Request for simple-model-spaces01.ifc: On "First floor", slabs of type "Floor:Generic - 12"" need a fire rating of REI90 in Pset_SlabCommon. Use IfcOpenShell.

First a look at what the model holds.

```python
import ifcopenshell
import ifcopenshell.util.element

model = ifcopenshell.open("simple-model-spaces01.ifc")
print(model.schema)
storey = next(s for s in model.by_type("IfcBuildingStorey") if s.Name == "First floor")
slabs = [e for e in ifcopenshell.util.element.get_decomposition(storey) if e.is_a("IfcSlab")]
seen = {}
for e in slabs:
    element_type = ifcopenshell.util.element.get_type(e)
    key = (element_type.Name if element_type != e and element_type else None, ifcopenshell.util.element.get_pset(e, "Pset_SlabCommon", "FireRating"))
    seen[key] = seen.get(key, 0) + 1
for (name, value), count in sorted(seen.items(), key=str):
    print(count, "x", name, "|", value)
```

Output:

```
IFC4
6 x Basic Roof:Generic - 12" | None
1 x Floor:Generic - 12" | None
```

```python
import ifcopenshell
import ifcopenshell.api.pset
import ifcopenshell.util.element

model = ifcopenshell.open("simple-model-spaces01.ifc")

storey = next(s for s in model.by_type("IfcBuildingStorey") if s.Name == "First floor")
slabs = [e for e in ifcopenshell.util.element.get_decomposition(storey) if e.is_a("IfcSlab")]

count = 0
for e in slabs:
    element_type = ifcopenshell.util.element.get_type(e)
    if element_type in (None, e) or element_type.Name != 'Floor:Generic - 12"':
        continue
    # add_pset returns the element's existing set when there is one.
    pset = ifcopenshell.api.pset.add_pset(model, product=e, name="Pset_SlabCommon")
    ifcopenshell.api.pset.edit_pset(model, pset=pset, properties={"FireRating": "REI90"})
    count += 1

print(count, "slabs updated")

model.write("simple-model-spaces01_rev.ifc")
```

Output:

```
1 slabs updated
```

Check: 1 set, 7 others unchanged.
